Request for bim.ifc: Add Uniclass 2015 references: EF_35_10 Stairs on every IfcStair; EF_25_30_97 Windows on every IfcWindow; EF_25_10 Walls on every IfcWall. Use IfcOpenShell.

First a look at what the model holds.

```python
import ifcopenshell

model = ifcopenshell.open("bim.ifc")
print(model.schema)
print("classifications:", [c.Name for c in model.by_type("IfcClassification")])
for ifc_class in ("IfcDoor", "IfcRoof", "IfcStair", "IfcWall", "IfcWindow"):
    print(ifc_class, len(model.by_type(ifc_class)))
```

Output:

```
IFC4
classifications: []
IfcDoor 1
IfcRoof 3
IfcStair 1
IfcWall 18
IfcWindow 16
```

```python
import ifcopenshell
import ifcopenshell.api.classification

model = ifcopenshell.open("bim.ifc")

system = ifcopenshell.api.classification.add_classification(model, classification="Uniclass 2015")

codes = {
    "IfcStair": ("EF_35_10", "Stairs"),
    "IfcWindow": ("EF_25_30_97", "Windows"),
    "IfcWall": ("EF_25_10", "Walls"),
}
for ifc_class, (code, name) in codes.items():
    products = model.by_type(ifc_class)
    ifcopenshell.api.classification.add_reference(
        model, products=products, classification=system, identification=code, name=name
    )
    print(code, len(products))

model.write("bim_updated.ifc")
```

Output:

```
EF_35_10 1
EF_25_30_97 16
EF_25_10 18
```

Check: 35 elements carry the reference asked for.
